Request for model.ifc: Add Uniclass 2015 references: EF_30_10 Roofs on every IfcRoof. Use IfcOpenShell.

First a look at what the model holds.

```python
import ifcopenshell

model = ifcopenshell.open("model.ifc")
print(model.schema)
print("classifications:", [c.Name for c in model.by_type("IfcClassification")])
for ifc_class in ("IfcDoor", "IfcRoof", "IfcStair", "IfcWall", "IfcWindow"):
    print(ifc_class, len(model.by_type(ifc_class)))
```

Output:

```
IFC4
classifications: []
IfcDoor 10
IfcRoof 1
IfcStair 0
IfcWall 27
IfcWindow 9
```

```python
import ifcopenshell
import ifcopenshell.api.classification

model = ifcopenshell.open("model.ifc")

system = ifcopenshell.api.classification.add_classification(model, classification="Uniclass 2015")

codes = {
    "IfcRoof": ("EF_30_10", "Roofs"),
}
for ifc_class, (code, name) in codes.items():
    products = model.by_type(ifc_class)
    ifcopenshell.api.classification.add_reference(
        model, products=products, classification=system, identification=code, name=name
    )
    print(code, len(products))

model.write("model_edited.ifc")
```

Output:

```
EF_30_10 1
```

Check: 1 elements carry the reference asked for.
